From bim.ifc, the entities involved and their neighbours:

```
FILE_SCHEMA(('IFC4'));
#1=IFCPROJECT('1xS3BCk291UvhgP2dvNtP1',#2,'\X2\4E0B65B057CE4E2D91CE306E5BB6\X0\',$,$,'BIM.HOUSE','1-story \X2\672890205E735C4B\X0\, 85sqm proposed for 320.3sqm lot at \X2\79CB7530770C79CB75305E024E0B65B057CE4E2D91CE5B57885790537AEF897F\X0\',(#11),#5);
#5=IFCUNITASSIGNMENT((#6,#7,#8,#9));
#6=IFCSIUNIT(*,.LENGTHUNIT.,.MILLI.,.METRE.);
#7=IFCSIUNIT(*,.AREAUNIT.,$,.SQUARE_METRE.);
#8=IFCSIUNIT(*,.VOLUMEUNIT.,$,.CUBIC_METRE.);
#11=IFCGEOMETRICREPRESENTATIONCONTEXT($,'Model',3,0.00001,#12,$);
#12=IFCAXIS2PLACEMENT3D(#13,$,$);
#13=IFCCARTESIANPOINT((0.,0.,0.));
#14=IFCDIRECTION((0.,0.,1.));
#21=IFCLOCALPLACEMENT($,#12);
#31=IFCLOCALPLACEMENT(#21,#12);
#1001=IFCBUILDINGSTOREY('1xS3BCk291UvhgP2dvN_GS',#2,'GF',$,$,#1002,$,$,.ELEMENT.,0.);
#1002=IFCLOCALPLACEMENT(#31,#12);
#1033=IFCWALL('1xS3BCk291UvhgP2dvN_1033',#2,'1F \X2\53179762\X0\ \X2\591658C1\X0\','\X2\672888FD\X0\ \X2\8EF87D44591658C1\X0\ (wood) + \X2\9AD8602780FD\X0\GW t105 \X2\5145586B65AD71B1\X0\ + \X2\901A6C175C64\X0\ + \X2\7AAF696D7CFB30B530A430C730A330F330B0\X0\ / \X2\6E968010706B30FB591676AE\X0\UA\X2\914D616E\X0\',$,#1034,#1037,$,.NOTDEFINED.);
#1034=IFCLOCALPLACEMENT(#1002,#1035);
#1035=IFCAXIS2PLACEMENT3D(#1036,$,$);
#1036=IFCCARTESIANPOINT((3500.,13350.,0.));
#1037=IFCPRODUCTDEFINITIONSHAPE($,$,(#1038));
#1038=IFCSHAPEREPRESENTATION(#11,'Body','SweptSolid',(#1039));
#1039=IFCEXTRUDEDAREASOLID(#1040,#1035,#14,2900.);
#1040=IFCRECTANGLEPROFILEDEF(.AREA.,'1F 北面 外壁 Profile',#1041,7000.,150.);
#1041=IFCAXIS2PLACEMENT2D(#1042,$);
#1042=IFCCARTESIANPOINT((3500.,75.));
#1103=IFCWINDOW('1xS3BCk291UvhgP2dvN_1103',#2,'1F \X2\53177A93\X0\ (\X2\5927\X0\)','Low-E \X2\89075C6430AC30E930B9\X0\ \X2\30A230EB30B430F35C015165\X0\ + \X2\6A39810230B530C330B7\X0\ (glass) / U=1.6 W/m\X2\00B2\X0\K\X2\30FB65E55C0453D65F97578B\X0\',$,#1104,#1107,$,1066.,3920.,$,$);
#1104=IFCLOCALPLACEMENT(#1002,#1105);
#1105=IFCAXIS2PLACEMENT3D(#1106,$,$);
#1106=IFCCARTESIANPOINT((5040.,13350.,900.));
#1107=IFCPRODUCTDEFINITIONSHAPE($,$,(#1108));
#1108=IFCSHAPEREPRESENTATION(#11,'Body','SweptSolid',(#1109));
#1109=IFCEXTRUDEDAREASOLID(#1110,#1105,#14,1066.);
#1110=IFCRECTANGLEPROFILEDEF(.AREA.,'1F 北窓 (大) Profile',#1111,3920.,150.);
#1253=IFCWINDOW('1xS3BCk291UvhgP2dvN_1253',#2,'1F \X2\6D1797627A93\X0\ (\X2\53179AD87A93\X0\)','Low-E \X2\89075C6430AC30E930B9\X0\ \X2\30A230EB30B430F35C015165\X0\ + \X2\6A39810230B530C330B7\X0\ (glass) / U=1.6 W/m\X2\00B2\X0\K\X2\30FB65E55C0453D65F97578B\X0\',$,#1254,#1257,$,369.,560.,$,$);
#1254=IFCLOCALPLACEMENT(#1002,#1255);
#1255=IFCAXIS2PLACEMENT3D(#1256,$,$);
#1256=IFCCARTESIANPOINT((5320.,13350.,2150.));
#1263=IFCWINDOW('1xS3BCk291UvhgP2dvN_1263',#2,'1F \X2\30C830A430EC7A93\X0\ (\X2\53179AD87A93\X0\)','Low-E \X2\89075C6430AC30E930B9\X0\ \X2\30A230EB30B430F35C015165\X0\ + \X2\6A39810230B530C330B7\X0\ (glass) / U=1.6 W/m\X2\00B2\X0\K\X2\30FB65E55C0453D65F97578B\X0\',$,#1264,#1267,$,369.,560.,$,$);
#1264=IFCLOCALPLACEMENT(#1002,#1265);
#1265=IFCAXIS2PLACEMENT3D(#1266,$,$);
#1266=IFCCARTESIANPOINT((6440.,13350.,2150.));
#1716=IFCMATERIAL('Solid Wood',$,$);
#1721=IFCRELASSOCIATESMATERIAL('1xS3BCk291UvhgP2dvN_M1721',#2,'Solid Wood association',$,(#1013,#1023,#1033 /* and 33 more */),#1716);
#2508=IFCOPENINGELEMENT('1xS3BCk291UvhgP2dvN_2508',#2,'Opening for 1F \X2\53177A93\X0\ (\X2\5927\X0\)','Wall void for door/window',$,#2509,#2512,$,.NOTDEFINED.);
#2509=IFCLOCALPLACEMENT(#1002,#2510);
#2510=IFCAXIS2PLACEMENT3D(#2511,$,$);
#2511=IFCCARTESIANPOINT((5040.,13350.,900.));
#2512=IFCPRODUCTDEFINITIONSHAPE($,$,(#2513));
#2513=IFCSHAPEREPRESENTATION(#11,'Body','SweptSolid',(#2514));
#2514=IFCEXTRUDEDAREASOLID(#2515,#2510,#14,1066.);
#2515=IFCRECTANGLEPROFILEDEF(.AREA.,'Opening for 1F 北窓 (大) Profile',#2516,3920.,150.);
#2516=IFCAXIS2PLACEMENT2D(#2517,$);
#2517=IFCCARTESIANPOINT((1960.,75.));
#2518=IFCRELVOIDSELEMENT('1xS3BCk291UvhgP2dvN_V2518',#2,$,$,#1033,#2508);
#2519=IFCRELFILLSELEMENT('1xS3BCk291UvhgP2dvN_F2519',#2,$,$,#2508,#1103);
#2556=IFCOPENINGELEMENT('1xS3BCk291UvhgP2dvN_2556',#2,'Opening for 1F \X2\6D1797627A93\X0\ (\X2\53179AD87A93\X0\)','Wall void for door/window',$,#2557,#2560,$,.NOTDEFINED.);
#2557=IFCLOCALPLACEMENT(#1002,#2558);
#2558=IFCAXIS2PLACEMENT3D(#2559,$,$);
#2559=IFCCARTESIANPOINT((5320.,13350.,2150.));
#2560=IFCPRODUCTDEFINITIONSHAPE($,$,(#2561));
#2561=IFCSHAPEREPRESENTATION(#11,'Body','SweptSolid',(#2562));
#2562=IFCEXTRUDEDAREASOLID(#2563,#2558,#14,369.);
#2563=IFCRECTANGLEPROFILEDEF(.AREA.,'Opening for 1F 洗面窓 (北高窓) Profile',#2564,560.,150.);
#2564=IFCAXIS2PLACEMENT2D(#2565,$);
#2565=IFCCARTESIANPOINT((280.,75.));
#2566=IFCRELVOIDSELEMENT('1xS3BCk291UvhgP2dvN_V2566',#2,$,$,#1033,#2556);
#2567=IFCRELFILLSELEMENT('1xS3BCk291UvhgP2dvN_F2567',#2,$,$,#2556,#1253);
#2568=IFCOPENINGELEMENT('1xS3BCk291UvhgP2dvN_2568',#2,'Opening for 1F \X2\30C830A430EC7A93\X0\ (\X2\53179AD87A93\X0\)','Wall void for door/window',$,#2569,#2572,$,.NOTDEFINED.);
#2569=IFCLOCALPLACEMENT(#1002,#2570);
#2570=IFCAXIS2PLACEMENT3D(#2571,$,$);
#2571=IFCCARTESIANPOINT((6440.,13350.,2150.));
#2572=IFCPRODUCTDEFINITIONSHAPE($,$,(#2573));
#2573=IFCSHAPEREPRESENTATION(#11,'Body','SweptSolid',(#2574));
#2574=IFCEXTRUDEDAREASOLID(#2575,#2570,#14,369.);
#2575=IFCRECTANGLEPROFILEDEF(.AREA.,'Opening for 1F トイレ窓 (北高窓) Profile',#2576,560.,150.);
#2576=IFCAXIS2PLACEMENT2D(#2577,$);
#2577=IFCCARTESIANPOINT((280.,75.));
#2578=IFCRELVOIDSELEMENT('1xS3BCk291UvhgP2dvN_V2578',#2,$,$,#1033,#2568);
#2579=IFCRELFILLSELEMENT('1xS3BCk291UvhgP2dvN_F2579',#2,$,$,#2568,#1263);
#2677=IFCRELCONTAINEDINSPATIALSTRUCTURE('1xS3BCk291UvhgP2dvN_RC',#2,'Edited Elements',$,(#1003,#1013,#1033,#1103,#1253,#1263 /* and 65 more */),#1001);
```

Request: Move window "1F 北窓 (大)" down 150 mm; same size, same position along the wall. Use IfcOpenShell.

```python
import numpy as np
import ifcopenshell
import ifcopenshell.api.geometry
import ifcopenshell.util.placement
import ifcopenshell.util.unit

model = ifcopenshell.open("bim.ifc")
unit_scale = ifcopenshell.util.unit.calculate_unit_scale(model)

window = model.by_guid("1xS3BCk291UvhgP2dvN_1103")
opening = window.FillsVoids[0].RelatingOpeningElement
dz = -150.0

shift = np.array([0.0, 0.0, dz])
# The window is not placed relative to its opening, so move both.
for product in (opening, window):
    matrix = ifcopenshell.util.placement.get_local_placement(product.ObjectPlacement)
    matrix[:3, 3] += shift
    ifcopenshell.api.geometry.edit_object_placement(model, product=product, matrix=matrix, is_si=False)

print(f"moved by {dz * unit_scale:+.3f} m")

model.write("bim-out.ifc")
```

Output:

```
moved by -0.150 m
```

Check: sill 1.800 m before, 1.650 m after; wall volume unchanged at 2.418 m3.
